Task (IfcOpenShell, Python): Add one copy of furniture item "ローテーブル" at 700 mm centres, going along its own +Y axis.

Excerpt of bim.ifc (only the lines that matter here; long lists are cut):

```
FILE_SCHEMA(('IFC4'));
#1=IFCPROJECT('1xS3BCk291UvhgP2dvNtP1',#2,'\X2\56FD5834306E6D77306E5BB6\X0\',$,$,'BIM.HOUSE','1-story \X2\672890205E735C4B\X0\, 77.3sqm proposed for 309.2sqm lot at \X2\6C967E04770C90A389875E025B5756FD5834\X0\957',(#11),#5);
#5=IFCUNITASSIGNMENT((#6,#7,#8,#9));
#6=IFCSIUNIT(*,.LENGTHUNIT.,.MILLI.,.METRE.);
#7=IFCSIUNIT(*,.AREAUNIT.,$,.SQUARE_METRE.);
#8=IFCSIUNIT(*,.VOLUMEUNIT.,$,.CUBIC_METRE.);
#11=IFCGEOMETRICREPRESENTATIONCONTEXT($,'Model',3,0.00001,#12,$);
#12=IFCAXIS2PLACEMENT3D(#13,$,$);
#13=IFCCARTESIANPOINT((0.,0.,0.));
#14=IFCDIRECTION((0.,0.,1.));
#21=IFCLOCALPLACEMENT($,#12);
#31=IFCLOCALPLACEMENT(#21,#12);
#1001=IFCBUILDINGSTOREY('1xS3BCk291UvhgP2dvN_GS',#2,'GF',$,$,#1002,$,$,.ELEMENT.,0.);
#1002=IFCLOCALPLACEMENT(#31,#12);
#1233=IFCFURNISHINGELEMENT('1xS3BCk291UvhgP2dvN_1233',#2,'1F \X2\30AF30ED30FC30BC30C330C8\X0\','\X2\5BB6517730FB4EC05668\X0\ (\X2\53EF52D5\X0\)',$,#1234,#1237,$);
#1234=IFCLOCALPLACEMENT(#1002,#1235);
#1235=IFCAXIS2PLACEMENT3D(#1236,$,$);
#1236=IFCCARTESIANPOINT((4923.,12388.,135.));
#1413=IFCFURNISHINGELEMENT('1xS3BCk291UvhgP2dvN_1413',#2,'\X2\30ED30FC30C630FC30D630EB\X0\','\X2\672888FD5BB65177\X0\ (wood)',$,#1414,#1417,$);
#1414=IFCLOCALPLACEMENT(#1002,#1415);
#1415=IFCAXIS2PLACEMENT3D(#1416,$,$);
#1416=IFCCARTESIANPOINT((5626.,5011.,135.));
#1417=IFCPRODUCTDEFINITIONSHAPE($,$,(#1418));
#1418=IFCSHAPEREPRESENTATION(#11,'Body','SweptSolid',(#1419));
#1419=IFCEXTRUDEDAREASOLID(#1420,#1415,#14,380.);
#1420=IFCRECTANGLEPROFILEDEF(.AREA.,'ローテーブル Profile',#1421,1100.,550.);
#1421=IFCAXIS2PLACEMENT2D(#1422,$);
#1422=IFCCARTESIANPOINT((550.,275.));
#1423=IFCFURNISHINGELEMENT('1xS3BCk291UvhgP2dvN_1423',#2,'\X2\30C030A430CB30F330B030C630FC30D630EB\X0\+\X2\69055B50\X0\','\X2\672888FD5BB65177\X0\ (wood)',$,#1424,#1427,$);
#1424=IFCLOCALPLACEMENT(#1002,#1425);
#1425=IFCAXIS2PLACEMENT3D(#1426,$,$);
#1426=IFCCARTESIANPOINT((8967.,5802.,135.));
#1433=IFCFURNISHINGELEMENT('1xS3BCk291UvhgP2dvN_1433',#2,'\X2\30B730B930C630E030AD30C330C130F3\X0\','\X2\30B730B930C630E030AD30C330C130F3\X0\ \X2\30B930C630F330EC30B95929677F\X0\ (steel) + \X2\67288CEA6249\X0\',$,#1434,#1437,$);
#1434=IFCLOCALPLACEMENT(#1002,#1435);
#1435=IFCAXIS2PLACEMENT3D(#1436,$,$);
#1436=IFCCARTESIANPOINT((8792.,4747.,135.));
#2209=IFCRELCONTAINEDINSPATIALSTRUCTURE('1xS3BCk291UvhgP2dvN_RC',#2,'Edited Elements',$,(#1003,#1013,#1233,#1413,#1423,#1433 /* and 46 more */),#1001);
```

```python
import ifcopenshell
import ifcopenshell.api.geometry
import ifcopenshell.api.root
import ifcopenshell.util.element
import ifcopenshell.util.placement

model = ifcopenshell.open("bim.ifc")


def reuse_history(source, copy):
    """copy_class also copies each property set's owner history, people and application; keep the originals."""
    for rel in copy.IsDefinedBy:
        if rel.is_a("IfcRelDefinesByProperties") and (history := rel.RelatingPropertyDefinition.OwnerHistory):
            rel.RelatingPropertyDefinition.OwnerHistory = source.OwnerHistory
            ifcopenshell.util.element.remove_deep2(model, history)


source = model.by_guid("1xS3BCk291UvhgP2dvN_1413")
base = ifcopenshell.util.placement.get_local_placement(source.ObjectPlacement)
step = base[:3, 1] * 700.0

for i in range(1, 2):
    copy = ifcopenshell.api.root.copy_class(model, product=source)
    copy.Representation = ifcopenshell.util.element.copy_deep(
        model, source.Representation, exclude=["IfcGeometricRepresentationContext", "IfcRepresentationMap"]
    )
    reuse_history(source, copy)
    matrix = base.copy()
    matrix[:3, 3] += i * step
    print("added at", matrix[:3, 3].round(3) + 0.0)
    ifcopenshell.api.geometry.edit_object_placement(model, product=copy, matrix=matrix, is_si=False)

model.write("bim_edited.ifc")
```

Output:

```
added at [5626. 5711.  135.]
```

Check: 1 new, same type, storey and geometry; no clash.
